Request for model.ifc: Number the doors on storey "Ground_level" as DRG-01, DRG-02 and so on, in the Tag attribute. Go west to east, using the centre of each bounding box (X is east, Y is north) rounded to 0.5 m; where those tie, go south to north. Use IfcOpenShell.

First a look at what the model holds.

```python
import ifcopenshell
import ifcopenshell.util.element
import ifcopenshell.util.placement

model = ifcopenshell.open("model.ifc")
print(model.schema)
storey = next(s for s in model.by_type("IfcBuildingStorey") if s.Name == "Ground_level")
doors = [e for e in ifcopenshell.util.element.get_decomposition(storey) if e.is_a("IfcDoor")]
for e in sorted(doors, key=lambda e: e.id()):
    origin = ifcopenshell.util.placement.get_local_placement(e.ObjectPlacement)[:3, 3]
    print(e.id(), e.Tag, e.Name, origin.round(2) + 0.0, sep=" | ")
```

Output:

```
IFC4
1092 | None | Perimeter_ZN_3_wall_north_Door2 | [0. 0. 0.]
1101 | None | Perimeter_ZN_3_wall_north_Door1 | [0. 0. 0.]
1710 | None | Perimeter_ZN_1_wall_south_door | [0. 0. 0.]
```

```python
import ifcopenshell
import ifcopenshell.geom
import ifcopenshell.util.element
import ifcopenshell.util.shape

model = ifcopenshell.open("model.ifc")
settings = ifcopenshell.geom.settings()
settings.set("use-world-coords", True)


def centre(element):
    shape = ifcopenshell.geom.create_shape(settings, element)
    return ifcopenshell.util.shape.get_bbox_centroid(shape.geometry)


storey = next(s for s in model.by_type("IfcBuildingStorey") if s.Name == "Ground_level")
doors = [e for e in ifcopenshell.util.element.get_decomposition(storey) if e.is_a("IfcDoor")]

# Insertion points can sit at a corner or the storey origin, so sort by the geometry (in metres).
centres = {e: centre(e) for e in doors}
doors.sort(key=lambda e: (round(centres[e][0] / 0.5), centres[e][1]))

for i, e in enumerate(doors, start=1):
    number = f"DRG-{i:02d}"
    e.Tag = number
    print(e.id(), number)

model.write("model-out.ifc")
```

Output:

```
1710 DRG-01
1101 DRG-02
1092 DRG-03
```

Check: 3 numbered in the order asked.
